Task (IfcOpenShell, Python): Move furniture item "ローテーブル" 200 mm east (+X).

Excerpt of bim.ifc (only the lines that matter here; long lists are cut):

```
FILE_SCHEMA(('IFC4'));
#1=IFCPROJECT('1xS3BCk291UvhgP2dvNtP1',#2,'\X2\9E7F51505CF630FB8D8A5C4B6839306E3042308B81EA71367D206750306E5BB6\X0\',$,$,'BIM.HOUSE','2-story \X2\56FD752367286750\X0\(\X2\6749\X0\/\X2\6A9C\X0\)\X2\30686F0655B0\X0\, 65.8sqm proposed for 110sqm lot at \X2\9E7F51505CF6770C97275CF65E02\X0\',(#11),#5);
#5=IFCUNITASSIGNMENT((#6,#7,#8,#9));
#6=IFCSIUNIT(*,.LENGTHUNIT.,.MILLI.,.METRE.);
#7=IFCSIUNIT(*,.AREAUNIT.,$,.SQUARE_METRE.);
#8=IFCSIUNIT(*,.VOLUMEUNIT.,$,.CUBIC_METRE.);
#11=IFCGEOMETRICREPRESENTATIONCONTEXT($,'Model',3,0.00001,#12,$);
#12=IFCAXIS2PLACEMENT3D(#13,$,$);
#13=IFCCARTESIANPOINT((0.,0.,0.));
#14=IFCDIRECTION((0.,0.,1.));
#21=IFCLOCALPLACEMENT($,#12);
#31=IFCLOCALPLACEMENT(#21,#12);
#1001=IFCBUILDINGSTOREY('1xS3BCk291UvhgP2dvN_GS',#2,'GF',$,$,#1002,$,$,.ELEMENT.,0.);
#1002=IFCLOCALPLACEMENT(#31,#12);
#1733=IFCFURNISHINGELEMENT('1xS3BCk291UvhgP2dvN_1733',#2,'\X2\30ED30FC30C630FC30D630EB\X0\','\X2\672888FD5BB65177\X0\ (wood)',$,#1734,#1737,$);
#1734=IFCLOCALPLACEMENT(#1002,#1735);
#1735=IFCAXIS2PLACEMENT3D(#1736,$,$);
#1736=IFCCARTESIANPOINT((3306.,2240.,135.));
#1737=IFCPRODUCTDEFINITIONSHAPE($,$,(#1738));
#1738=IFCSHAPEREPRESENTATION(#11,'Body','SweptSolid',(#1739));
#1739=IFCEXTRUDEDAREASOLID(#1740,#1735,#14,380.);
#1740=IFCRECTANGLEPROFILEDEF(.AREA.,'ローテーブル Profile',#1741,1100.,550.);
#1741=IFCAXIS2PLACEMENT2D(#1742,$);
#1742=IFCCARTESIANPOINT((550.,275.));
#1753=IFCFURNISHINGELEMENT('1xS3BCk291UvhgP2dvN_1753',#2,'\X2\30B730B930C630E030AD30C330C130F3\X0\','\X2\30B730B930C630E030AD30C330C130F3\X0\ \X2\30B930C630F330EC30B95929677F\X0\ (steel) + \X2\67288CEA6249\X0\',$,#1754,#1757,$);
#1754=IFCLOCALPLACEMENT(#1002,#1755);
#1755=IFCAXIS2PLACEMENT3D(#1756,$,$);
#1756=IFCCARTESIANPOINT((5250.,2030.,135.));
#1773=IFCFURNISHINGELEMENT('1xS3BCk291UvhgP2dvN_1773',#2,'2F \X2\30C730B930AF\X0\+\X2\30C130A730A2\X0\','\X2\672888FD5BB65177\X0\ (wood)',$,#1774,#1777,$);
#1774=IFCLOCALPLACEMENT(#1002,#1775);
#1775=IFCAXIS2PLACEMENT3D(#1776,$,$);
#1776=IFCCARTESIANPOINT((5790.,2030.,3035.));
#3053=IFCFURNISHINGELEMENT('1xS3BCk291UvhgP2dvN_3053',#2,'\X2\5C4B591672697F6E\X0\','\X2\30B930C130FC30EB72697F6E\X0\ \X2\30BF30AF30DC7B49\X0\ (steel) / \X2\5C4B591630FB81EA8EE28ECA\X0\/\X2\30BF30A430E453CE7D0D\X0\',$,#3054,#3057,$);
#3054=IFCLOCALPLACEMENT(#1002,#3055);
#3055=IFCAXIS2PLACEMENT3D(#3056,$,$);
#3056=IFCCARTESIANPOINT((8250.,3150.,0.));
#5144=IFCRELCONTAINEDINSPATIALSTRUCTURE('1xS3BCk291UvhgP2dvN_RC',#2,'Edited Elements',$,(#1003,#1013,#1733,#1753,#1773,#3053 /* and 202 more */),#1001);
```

```python
import ifcopenshell
import ifcopenshell.api.geometry
import ifcopenshell.util.placement
import ifcopenshell.util.unit

model = ifcopenshell.open("bim.ifc")
unit_scale = ifcopenshell.util.unit.calculate_unit_scale(model)

item = model.by_id(1733)
matrix = ifcopenshell.util.placement.get_local_placement(item.ObjectPlacement)
matrix[0, 3] += 0.2 / unit_scale
ifcopenshell.api.geometry.edit_object_placement(model, product=item, matrix=matrix, is_si=False)

print(ifcopenshell.util.placement.get_local_placement(item.ObjectPlacement).round(3) + 0.0)

model.write("bim_edited.ifc")
```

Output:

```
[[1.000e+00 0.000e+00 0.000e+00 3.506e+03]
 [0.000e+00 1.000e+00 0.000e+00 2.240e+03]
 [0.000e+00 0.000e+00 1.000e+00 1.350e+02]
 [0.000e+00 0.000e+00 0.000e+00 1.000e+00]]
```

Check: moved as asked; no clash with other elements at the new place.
